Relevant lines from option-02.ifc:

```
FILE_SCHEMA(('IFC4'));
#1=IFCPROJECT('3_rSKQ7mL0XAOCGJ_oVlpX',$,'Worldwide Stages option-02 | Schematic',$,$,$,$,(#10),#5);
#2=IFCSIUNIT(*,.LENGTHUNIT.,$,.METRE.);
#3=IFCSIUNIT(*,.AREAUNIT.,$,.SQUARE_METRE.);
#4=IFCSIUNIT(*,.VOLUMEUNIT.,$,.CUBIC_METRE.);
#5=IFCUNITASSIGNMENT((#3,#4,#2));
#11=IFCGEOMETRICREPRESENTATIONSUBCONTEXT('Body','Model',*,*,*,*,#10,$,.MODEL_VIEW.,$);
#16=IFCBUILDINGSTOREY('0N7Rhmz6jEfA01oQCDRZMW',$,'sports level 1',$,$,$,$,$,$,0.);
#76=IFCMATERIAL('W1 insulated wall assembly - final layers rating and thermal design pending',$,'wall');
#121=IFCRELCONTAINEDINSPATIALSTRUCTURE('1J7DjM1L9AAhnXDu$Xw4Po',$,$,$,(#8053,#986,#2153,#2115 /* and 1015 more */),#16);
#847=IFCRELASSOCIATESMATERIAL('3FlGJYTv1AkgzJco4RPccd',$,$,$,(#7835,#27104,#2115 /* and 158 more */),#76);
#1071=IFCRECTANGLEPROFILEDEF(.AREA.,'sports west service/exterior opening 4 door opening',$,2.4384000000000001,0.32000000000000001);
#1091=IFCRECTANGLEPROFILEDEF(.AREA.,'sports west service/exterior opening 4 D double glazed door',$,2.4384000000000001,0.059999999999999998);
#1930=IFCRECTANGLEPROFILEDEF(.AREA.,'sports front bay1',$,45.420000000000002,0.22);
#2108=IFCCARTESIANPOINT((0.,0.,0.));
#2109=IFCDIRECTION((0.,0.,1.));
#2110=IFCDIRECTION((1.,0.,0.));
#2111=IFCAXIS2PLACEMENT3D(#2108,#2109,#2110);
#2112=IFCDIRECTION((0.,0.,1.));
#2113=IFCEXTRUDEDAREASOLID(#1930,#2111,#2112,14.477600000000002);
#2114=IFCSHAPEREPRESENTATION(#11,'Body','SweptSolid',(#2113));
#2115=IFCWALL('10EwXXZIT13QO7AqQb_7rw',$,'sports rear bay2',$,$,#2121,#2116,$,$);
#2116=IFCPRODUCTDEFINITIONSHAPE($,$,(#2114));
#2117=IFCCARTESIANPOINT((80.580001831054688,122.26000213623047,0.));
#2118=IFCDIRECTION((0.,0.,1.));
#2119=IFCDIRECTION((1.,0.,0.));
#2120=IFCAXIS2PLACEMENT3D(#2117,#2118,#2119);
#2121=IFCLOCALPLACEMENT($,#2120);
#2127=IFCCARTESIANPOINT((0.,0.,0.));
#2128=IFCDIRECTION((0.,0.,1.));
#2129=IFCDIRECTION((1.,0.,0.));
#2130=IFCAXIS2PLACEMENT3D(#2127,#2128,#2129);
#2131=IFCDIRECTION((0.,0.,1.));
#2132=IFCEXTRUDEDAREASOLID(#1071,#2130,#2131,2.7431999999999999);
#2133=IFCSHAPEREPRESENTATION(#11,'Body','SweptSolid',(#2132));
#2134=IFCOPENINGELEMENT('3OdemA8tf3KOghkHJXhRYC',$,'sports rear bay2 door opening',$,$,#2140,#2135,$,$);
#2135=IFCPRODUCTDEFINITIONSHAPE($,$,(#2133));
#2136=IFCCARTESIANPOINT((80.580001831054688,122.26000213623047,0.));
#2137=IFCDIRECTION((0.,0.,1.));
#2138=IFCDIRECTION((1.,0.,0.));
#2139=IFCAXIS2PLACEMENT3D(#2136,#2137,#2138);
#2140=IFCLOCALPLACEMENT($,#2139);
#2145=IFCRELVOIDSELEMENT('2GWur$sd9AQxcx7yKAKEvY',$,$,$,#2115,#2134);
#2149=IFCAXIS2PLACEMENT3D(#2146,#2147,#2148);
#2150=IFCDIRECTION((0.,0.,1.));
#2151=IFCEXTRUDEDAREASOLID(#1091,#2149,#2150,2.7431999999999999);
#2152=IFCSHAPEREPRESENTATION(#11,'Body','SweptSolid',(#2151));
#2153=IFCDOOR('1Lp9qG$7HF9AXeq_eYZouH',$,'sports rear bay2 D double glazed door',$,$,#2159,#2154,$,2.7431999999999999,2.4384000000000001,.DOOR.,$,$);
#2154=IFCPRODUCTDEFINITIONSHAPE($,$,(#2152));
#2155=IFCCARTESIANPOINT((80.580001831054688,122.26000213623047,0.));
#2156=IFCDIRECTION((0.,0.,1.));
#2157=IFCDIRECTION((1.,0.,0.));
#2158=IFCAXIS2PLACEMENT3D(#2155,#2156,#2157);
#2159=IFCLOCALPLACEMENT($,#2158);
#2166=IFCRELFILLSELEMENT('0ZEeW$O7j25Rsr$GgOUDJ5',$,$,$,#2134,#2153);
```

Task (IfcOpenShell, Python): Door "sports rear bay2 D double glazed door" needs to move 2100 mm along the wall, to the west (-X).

```python
import ifcopenshell
import ifcopenshell.api.geometry
import ifcopenshell.util.placement
import ifcopenshell.util.unit

model = ifcopenshell.open("option-02.ifc")
unit_scale = ifcopenshell.util.unit.calculate_unit_scale(model)

door = model.by_guid("1Lp9qG$7HF9AXeq_eYZouH")
opening = door.FillsVoids[0].RelatingOpeningElement
wall = opening.VoidsElements[0].RelatingBuildingElement

wall_matrix = ifcopenshell.util.placement.get_local_placement(wall.ObjectPlacement)
shift = wall_matrix[:3, 0] * -2.1 / unit_scale
before = ifcopenshell.util.placement.get_local_placement(door.ObjectPlacement)[:3, 3].copy()

# The door is not placed relative to its opening, so move both.
for product in (opening, door):
    matrix = ifcopenshell.util.placement.get_local_placement(product.ObjectPlacement)
    matrix[:3, 3] += shift
    ifcopenshell.api.geometry.edit_object_placement(model, product=product, matrix=matrix, is_si=False)

after = ifcopenshell.util.placement.get_local_placement(door.ObjectPlacement)[:3, 3]
print("door moved by", (after - before).round(3) + 0.0)

model.write("option-02_edited.ifc")
```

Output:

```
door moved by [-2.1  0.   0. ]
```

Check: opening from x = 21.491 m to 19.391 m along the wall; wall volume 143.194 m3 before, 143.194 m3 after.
